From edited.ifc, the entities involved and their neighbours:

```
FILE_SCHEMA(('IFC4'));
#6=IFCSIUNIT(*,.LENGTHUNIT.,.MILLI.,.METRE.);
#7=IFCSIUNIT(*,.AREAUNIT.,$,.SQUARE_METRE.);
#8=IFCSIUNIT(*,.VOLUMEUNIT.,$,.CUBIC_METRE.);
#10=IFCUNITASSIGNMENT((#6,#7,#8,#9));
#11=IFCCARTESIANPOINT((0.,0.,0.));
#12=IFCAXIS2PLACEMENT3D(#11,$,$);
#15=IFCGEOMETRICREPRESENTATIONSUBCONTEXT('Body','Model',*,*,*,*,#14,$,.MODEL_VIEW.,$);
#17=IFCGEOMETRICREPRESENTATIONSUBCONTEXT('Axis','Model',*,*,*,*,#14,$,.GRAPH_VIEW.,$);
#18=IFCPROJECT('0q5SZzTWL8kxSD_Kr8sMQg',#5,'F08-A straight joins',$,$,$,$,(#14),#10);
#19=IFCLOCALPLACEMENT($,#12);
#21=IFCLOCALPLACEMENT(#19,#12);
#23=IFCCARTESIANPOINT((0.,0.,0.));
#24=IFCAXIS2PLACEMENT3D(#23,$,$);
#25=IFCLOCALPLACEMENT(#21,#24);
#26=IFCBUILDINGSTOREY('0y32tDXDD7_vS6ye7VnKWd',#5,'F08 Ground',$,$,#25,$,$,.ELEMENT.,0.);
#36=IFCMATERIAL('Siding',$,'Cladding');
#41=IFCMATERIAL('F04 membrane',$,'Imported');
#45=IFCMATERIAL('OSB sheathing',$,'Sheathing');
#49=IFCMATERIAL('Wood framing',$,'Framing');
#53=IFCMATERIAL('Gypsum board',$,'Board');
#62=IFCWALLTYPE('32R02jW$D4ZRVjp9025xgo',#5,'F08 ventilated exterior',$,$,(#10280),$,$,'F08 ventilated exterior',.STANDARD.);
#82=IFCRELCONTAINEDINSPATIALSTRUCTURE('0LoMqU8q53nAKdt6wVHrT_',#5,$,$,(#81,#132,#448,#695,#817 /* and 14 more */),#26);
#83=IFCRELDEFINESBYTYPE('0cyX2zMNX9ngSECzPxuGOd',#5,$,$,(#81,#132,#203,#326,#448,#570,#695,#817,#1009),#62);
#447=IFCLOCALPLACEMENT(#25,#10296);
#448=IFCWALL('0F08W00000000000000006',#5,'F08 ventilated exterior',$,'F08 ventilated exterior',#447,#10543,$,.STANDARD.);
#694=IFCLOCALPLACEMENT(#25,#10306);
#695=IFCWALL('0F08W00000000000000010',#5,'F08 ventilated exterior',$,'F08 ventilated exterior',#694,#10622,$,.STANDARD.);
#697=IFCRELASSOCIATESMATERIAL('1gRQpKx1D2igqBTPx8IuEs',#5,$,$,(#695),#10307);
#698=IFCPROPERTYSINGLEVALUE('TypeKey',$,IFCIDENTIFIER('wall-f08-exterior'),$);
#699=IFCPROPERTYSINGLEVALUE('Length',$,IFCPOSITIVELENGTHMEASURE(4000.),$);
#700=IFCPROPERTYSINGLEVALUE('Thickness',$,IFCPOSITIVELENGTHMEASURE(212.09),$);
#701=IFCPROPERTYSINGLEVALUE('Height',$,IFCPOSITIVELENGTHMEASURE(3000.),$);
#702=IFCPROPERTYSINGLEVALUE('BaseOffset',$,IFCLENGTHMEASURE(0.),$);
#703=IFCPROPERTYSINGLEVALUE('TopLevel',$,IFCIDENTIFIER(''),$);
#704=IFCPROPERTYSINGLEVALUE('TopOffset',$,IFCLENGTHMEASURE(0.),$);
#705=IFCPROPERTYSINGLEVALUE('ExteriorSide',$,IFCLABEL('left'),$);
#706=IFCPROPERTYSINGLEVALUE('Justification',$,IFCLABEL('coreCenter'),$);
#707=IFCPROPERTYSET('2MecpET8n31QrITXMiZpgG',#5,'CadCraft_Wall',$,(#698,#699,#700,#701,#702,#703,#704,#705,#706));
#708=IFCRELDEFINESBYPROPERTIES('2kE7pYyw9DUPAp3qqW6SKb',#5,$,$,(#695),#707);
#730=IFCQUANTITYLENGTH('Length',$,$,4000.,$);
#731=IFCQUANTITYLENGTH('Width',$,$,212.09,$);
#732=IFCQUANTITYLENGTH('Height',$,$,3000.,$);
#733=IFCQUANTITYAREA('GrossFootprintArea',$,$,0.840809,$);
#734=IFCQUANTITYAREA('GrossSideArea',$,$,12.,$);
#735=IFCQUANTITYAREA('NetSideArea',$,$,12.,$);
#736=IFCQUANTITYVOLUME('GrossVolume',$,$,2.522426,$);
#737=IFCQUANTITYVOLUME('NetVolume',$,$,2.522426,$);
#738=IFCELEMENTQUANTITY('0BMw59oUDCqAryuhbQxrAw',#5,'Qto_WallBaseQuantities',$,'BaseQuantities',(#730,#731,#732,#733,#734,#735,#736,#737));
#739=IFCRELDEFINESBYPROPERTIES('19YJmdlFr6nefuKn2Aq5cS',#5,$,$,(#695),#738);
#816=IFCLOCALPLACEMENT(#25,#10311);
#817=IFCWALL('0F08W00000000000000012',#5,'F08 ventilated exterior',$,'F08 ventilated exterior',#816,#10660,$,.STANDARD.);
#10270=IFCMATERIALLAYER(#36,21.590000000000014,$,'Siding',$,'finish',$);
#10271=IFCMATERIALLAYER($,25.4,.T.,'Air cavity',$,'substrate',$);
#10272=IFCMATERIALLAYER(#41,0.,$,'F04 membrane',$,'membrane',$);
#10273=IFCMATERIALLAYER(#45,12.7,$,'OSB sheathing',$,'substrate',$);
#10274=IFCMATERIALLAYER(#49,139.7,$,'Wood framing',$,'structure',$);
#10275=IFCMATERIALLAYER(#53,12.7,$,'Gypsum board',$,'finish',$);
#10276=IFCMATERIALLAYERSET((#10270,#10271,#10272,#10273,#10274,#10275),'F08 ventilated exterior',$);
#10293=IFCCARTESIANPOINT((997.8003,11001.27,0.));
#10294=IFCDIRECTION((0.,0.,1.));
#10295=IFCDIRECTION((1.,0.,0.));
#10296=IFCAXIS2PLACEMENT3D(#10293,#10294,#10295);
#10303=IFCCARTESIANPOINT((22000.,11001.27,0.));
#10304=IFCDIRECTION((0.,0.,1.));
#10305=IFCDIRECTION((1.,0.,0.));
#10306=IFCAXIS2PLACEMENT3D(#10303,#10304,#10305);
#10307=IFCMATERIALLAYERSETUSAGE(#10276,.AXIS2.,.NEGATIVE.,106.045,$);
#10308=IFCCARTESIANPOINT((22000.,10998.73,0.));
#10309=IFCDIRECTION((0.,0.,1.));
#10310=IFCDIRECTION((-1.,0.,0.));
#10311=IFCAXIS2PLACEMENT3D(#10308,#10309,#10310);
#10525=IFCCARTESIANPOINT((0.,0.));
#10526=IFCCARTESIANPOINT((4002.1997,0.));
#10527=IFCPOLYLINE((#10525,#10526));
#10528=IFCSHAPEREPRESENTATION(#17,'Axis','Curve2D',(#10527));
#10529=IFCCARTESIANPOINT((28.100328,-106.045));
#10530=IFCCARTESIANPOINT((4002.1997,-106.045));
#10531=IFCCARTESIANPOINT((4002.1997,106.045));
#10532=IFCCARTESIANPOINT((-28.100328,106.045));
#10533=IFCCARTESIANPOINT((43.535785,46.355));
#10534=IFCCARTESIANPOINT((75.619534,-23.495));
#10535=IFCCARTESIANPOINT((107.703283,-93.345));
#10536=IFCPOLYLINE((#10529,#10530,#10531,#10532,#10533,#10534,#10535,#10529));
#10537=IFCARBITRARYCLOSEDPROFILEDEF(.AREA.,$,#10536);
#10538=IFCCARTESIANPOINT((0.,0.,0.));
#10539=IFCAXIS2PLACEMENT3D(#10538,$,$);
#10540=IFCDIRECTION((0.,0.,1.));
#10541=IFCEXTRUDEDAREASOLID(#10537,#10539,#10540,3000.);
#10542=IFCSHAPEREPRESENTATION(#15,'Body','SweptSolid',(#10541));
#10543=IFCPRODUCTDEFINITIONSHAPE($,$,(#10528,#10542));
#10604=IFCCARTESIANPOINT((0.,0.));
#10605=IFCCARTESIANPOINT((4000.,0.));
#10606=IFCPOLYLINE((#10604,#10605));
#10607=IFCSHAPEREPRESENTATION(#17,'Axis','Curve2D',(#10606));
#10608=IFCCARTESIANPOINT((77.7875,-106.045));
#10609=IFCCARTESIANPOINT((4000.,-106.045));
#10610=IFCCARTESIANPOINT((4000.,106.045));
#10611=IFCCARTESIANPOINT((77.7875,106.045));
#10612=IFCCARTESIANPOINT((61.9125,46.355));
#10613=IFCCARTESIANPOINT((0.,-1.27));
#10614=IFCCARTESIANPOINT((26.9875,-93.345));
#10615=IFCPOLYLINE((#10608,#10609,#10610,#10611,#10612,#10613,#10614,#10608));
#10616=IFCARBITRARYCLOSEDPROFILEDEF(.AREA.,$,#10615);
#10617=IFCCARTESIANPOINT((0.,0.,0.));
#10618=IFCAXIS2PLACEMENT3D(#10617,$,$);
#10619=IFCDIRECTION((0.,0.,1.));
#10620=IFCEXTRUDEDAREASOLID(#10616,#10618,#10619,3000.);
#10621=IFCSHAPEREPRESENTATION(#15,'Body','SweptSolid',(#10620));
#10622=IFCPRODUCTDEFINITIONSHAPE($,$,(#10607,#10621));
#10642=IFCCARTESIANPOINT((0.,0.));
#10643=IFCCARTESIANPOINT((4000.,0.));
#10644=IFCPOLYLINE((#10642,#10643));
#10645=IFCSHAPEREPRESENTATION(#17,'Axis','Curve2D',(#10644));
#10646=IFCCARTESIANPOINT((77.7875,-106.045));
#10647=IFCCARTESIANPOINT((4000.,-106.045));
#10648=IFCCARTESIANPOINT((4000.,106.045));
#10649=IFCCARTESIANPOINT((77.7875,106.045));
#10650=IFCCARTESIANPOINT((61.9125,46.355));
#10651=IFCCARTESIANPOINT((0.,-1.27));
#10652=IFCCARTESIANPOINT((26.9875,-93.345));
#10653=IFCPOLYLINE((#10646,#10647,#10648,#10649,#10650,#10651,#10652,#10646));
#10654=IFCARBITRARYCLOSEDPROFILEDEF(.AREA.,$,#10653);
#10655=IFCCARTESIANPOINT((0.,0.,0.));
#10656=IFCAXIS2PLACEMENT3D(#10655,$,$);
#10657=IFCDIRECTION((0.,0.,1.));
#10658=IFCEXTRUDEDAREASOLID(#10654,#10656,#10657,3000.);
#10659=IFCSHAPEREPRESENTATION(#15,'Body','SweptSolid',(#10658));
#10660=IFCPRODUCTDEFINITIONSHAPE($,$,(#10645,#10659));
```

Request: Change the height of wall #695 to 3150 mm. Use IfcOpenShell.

```python
import ifcopenshell
import ifcopenshell.api.pset
import ifcopenshell.geom
import ifcopenshell.util.element
import ifcopenshell.util.representation
import ifcopenshell.util.shape
import ifcopenshell.util.unit

model = ifcopenshell.open("edited.ifc")
unit_scale = ifcopenshell.util.unit.calculate_unit_scale(model)
area_scale = ifcopenshell.util.unit.calculate_unit_scale(model, "AREAUNIT")
volume_scale = ifcopenshell.util.unit.calculate_unit_scale(model, "VOLUMEUNIT")
settings = ifcopenshell.geom.settings()


def volume(element):
    """Net volume in cubic metres, openings subtracted."""
    shape = ifcopenshell.geom.create_shape(settings, element)
    return ifcopenshell.util.shape.get_volume(shape.geometry)


wall = model.by_guid("0F08W00000000000000010")
before = volume(wall)

body = ifcopenshell.util.representation.get_representation(wall, "Model", "Body")
solid = body.Items[0]
old_height = solid.Depth
solid.Depth = 3.15 / unit_scale
after = volume(wall)
thickness = 0.2121  # wall thickness in metres

# Update the stored height, areas and volumes.
pset = model.by_id(ifcopenshell.util.element.get_pset(wall, "CadCraft_Wall", should_inherit=False)["id"])
ifcopenshell.api.pset.edit_pset(model, pset=pset, properties={
    "Height": model.create_entity("IfcPositiveLengthMeasure", solid.Depth),
})
qto = model.by_id(ifcopenshell.util.element.get_pset(wall, "Qto_WallBaseQuantities", should_inherit=False)["id"])
ifcopenshell.api.pset.edit_qto(model, qto=qto, properties={
    "Height": solid.Depth,
    "GrossSideArea": ifcopenshell.util.element.get_pset(wall, "Qto_WallBaseQuantities", "GrossSideArea") * solid.Depth / old_height,
    "NetSideArea": after / thickness / area_scale,
    "GrossVolume": ifcopenshell.util.element.get_pset(wall, "Qto_WallBaseQuantities", "GrossVolume") * solid.Depth / old_height,
    "NetVolume": after / volume_scale,
})

print(f"height {old_height:g} -> {solid.Depth:g}, volume {before:.3f} -> {after:.3f} m3")

model.write("edited_v2.ifc")
```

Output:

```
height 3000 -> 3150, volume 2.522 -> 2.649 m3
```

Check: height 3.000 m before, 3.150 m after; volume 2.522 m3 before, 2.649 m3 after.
